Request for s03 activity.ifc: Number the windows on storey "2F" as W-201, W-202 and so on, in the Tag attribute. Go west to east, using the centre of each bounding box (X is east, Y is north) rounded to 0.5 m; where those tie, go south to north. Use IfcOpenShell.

First a look at what the model holds.

```python
import ifcopenshell
import ifcopenshell.util.element
import ifcopenshell.util.placement

model = ifcopenshell.open("s03 activity.ifc")
print(model.schema)
storey = next(s for s in model.by_type("IfcBuildingStorey") if s.Name == "2F")
windows = [e for e in ifcopenshell.util.element.get_decomposition(storey) if e.is_a("IfcWindow")]
for e in sorted(windows, key=lambda e: e.id()):
    origin = ifcopenshell.util.placement.get_local_placement(e.ObjectPlacement)[:3, 3]
    print(e.id(), e.Tag, e.Name, origin.round(2) + 0.0, sep=" | ")
```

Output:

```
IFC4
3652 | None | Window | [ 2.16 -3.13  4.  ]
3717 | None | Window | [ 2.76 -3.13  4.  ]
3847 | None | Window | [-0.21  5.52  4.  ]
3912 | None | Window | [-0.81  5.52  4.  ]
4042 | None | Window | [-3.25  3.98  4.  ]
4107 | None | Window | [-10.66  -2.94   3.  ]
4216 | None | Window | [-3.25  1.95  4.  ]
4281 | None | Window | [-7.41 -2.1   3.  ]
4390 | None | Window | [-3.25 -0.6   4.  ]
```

```python
import ifcopenshell
import ifcopenshell.geom
import ifcopenshell.util.element
import ifcopenshell.util.shape

model = ifcopenshell.open("s03 activity.ifc")
settings = ifcopenshell.geom.settings()
settings.set("use-world-coords", True)


def centre(element):
    shape = ifcopenshell.geom.create_shape(settings, element)
    return ifcopenshell.util.shape.get_bbox_centroid(shape.geometry)


storey = next(s for s in model.by_type("IfcBuildingStorey") if s.Name == "2F")
windows = [e for e in ifcopenshell.util.element.get_decomposition(storey) if e.is_a("IfcWindow")]

# Insertion points can sit at a corner or the storey origin, so sort by the geometry (in metres).
centres = {e: centre(e) for e in windows}
windows.sort(key=lambda e: (round(centres[e][0] / 0.5), centres[e][1]))

for i, e in enumerate(windows, start=1):
    number = f"W-2{i:02d}"
    e.Tag = number
    print(e.id(), number)

model.write("s03 activity_v2.ifc")
```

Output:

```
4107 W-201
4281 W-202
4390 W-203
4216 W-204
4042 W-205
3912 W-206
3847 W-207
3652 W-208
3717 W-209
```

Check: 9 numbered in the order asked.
